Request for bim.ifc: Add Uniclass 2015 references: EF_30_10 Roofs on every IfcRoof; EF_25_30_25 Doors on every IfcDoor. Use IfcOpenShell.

First a look at what the model holds.

```python
import ifcopenshell

model = ifcopenshell.open("bim.ifc")
print(model.schema)
print("classifications:", [c.Name for c in model.by_type("IfcClassification")])
for ifc_class in ("IfcDoor", "IfcRoof", "IfcStair", "IfcWall", "IfcWindow"):
    print(ifc_class, len(model.by_type(ifc_class)))
```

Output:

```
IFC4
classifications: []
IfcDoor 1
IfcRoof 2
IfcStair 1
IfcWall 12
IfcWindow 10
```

```python
import ifcopenshell
import ifcopenshell.api.classification

model = ifcopenshell.open("bim.ifc")

system = ifcopenshell.api.classification.add_classification(model, classification="Uniclass 2015")

codes = {
    "IfcRoof": ("EF_30_10", "Roofs"),
    "IfcDoor": ("EF_25_30_25", "Doors"),
}
for ifc_class, (code, name) in codes.items():
    products = model.by_type(ifc_class)
    ifcopenshell.api.classification.add_reference(
        model, products=products, classification=system, identification=code, name=name
    )
    print(code, len(products))

model.write("bim_v2.ifc")
```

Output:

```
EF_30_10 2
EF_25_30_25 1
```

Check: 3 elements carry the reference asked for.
